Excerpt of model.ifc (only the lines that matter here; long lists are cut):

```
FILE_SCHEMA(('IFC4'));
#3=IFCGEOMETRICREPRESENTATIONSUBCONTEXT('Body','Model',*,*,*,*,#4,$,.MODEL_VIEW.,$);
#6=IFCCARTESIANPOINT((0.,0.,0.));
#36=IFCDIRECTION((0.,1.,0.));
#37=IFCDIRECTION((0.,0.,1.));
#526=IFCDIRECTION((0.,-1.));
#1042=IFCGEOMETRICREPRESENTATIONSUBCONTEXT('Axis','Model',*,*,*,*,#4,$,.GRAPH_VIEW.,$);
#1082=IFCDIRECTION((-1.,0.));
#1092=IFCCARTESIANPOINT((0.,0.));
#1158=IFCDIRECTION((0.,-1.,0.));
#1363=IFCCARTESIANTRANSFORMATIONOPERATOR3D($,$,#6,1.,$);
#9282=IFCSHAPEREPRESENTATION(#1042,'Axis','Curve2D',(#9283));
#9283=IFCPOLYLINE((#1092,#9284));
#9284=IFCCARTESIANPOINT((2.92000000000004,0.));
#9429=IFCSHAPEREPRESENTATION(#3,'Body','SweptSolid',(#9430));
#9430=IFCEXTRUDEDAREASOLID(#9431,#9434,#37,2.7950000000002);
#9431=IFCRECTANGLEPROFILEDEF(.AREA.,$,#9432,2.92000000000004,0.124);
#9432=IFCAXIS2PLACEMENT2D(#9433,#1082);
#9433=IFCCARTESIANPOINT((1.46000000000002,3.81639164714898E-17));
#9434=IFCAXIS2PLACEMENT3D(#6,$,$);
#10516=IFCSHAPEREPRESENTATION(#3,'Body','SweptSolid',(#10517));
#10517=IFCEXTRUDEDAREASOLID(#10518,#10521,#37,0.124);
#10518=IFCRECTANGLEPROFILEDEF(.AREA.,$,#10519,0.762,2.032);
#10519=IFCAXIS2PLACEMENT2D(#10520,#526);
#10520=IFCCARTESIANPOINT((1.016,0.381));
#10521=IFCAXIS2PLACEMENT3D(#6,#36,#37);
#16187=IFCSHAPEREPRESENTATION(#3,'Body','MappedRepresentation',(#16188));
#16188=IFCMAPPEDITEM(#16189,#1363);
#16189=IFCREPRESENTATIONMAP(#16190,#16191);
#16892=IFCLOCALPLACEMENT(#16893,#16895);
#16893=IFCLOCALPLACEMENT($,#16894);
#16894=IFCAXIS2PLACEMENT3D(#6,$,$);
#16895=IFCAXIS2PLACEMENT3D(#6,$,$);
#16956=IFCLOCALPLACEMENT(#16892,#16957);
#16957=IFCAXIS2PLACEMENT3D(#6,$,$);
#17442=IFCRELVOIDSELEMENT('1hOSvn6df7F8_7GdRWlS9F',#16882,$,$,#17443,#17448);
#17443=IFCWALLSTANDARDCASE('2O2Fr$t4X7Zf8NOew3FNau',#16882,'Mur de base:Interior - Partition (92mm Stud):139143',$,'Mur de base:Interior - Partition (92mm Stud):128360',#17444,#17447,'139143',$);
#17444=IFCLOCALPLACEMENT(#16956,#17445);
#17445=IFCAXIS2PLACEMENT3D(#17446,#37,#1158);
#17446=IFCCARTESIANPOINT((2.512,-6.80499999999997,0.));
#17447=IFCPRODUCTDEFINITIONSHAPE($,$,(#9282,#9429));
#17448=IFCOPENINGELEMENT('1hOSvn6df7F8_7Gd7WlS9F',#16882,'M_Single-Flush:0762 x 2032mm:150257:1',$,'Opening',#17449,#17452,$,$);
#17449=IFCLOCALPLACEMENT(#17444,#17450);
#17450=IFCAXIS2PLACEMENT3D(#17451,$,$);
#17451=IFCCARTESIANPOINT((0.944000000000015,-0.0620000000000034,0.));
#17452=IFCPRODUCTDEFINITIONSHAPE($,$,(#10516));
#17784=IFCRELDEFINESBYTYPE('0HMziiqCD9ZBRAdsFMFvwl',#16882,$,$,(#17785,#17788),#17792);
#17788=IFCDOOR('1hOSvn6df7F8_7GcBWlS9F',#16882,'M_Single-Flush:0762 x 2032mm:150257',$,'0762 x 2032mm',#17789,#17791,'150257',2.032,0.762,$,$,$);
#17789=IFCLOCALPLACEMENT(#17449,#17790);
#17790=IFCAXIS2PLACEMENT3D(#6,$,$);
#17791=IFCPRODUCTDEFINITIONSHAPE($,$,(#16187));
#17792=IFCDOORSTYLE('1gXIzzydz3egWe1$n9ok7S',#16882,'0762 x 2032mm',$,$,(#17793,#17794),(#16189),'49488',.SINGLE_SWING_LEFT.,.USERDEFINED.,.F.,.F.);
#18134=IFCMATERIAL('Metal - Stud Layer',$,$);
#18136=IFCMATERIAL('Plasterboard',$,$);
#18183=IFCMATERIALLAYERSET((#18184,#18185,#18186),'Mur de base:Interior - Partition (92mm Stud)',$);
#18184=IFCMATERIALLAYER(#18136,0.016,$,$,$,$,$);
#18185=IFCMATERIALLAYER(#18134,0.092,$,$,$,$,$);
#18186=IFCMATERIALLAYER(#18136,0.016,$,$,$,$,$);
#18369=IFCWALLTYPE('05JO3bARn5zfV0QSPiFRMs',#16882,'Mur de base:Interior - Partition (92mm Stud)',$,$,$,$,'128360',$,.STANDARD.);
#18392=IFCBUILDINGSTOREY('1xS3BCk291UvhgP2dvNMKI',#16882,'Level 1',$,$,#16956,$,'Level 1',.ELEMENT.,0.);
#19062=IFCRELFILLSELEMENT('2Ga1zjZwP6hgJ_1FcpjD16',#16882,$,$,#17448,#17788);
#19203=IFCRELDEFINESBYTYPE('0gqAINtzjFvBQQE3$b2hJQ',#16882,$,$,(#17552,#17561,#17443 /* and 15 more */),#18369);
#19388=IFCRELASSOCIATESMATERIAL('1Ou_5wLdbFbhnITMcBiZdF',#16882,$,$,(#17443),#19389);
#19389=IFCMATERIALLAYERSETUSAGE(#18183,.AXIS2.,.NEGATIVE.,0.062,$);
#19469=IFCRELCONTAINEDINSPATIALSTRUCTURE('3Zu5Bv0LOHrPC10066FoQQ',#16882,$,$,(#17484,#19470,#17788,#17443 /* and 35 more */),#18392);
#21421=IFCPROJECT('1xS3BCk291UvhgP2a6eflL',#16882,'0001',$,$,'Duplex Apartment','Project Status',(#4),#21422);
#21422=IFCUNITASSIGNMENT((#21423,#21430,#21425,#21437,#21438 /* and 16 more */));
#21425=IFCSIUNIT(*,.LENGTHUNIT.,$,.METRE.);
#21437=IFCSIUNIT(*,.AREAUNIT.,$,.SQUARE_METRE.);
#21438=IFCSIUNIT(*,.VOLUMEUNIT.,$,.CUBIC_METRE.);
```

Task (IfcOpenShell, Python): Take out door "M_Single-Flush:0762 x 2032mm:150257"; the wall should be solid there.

```python
import ifcopenshell
import ifcopenshell.api.feature
import ifcopenshell.api.root
import ifcopenshell.geom
import ifcopenshell.util.shape

model = ifcopenshell.open("model.ifc")
settings = ifcopenshell.geom.settings()


def volume(element):
    """Net volume in cubic metres, openings subtracted."""
    shape = ifcopenshell.geom.create_shape(settings, element)
    return ifcopenshell.util.shape.get_volume(shape.geometry)


door = model.by_guid("1hOSvn6df7F8_7GcBWlS9F")
opening = door.FillsVoids[0].RelatingOpeningElement
wall = opening.VoidsElements[0].RelatingBuildingElement
before = volume(wall)

ifcopenshell.api.root.remove_product(model, product=door)
ifcopenshell.api.feature.remove_feature(model, feature=opening)

after = volume(wall)

print(f"wall volume {before:.3f} -> {after:.3f} m3")

model.write("model_v2.ifc")
```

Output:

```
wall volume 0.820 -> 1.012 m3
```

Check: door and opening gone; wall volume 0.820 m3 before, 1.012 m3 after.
